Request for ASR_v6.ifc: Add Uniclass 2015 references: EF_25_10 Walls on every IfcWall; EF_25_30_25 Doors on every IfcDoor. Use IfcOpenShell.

First a look at what the model holds.

```python
import ifcopenshell

model = ifcopenshell.open("ASR_v6.ifc")
print(model.schema)
print("classifications:", [c.Name for c in model.by_type("IfcClassification")])
for ifc_class in ("IfcDoor", "IfcRoof", "IfcStair", "IfcWall", "IfcWindow"):
    print(ifc_class, len(model.by_type(ifc_class)))
```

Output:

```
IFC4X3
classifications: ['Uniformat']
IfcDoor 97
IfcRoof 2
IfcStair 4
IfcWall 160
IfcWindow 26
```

```python
import ifcopenshell
import ifcopenshell.api.classification

model = ifcopenshell.open("ASR_v6.ifc")

system = ifcopenshell.api.classification.add_classification(model, classification="Uniclass 2015")

codes = {
    "IfcWall": ("EF_25_10", "Walls"),
    "IfcDoor": ("EF_25_30_25", "Doors"),
}
for ifc_class, (code, name) in codes.items():
    products = model.by_type(ifc_class)
    ifcopenshell.api.classification.add_reference(
        model, products=products, classification=system, identification=code, name=name
    )
    print(code, len(products))

model.write("ASR_v6_edited.ifc")
```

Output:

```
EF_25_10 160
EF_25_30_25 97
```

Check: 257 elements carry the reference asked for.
